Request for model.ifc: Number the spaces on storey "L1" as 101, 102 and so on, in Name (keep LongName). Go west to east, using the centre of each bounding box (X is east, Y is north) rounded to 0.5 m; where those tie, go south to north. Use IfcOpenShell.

First a look at what the model holds.

```python
import ifcopenshell
import ifcopenshell.util.element
import ifcopenshell.util.placement

model = ifcopenshell.open("model.ifc")
print(model.schema)
storey = next(s for s in model.by_type("IfcBuildingStorey") if s.Name == "L1")
spaces = [e for e in ifcopenshell.util.element.get_decomposition(storey) if e.is_a("IfcSpace")]
for e in sorted(spaces, key=lambda e: e.id()):
    origin = ifcopenshell.util.placement.get_local_placement(e.ObjectPlacement)[:3, 3]
    print(e.id(), e.Name, e.LongName, origin.round(2) + 0.0, sep=" | ")
```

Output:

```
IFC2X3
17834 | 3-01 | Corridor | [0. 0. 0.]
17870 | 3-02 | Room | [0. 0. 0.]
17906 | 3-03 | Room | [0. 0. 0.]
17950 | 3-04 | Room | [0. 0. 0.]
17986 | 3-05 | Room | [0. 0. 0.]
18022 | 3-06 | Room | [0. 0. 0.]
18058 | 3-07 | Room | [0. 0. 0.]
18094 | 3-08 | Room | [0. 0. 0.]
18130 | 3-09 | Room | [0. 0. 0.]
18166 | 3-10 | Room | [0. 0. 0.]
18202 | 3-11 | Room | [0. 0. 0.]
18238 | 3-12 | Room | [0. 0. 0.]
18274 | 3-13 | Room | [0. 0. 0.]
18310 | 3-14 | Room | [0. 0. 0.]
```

```python
import ifcopenshell
import ifcopenshell.geom
import ifcopenshell.util.element
import ifcopenshell.util.shape

model = ifcopenshell.open("model.ifc")
settings = ifcopenshell.geom.settings()
settings.set("use-world-coords", True)


def centre(element):
    shape = ifcopenshell.geom.create_shape(settings, element)
    return ifcopenshell.util.shape.get_bbox_centroid(shape.geometry)


storey = next(s for s in model.by_type("IfcBuildingStorey") if s.Name == "L1")
spaces = [e for e in ifcopenshell.util.element.get_decomposition(storey) if e.is_a("IfcSpace")]

# Insertion points can sit at a corner or the storey origin, so sort by the geometry (in metres).
centres = {e: centre(e) for e in spaces}
spaces.sort(key=lambda e: (round(centres[e][0] / 0.5), centres[e][1]))

for i, e in enumerate(spaces, start=1):
    number = f"1{i:02d}"
    e.Name = number
    print(e.id(), number)

model.write("model_v2.ifc")
```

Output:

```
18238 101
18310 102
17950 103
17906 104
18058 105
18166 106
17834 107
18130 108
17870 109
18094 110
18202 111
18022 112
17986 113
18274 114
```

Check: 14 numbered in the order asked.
